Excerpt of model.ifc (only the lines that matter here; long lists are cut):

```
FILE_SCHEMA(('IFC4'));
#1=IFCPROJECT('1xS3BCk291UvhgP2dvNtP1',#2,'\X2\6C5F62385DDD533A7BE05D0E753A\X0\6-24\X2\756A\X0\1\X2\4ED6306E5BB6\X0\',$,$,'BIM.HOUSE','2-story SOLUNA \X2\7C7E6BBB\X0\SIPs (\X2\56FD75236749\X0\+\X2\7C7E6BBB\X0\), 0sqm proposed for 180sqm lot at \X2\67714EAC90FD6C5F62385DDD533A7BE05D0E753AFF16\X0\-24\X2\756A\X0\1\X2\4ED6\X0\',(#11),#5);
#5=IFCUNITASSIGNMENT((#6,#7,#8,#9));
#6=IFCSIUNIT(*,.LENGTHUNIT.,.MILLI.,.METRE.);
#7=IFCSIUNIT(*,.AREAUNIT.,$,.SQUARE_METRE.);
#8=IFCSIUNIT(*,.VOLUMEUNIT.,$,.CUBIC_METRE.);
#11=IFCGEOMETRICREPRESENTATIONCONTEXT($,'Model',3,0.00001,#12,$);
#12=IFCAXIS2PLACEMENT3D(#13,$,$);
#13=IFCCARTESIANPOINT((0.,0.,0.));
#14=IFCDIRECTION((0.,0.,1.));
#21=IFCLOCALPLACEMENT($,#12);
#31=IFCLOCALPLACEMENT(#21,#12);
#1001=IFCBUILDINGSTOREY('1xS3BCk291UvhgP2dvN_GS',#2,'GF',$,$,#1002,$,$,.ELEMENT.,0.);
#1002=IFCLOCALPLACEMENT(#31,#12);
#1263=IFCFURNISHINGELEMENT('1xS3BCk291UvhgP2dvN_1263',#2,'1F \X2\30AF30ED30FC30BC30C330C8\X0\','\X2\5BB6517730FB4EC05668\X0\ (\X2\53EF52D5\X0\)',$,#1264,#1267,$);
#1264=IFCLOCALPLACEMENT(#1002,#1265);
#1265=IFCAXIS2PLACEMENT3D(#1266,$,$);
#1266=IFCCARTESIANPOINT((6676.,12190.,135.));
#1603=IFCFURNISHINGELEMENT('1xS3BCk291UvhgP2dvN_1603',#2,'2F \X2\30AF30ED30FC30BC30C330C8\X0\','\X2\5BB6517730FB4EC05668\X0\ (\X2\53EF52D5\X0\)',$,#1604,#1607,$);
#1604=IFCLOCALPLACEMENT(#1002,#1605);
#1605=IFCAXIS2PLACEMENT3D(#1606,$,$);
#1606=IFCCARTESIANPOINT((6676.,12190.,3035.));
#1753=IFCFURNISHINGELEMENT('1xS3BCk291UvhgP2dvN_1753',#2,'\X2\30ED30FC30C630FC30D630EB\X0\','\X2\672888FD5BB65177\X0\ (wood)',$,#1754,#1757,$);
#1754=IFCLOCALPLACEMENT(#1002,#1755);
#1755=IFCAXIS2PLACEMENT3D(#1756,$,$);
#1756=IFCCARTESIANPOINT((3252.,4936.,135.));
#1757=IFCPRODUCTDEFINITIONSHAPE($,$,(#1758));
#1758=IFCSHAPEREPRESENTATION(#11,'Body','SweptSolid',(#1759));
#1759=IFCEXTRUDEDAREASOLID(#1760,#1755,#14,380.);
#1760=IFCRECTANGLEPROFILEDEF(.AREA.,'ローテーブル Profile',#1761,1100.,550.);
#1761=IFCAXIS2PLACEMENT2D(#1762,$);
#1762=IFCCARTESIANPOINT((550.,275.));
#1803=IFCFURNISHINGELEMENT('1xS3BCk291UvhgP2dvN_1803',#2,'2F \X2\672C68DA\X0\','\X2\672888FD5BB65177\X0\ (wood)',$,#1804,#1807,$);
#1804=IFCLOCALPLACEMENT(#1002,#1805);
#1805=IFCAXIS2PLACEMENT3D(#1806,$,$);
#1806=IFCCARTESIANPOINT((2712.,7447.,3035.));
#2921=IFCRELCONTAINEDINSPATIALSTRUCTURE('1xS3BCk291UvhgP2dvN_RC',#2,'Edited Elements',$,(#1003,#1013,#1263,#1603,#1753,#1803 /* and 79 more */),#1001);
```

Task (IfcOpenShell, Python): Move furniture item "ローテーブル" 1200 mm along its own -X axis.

```python
import ifcopenshell
import ifcopenshell.api.geometry
import ifcopenshell.util.placement
import ifcopenshell.util.unit

model = ifcopenshell.open("model.ifc")
unit_scale = ifcopenshell.util.unit.calculate_unit_scale(model)

item = model.by_guid("1xS3BCk291UvhgP2dvN_1753")
matrix = ifcopenshell.util.placement.get_local_placement(item.ObjectPlacement)
matrix[:3, 3] -= matrix[:3, 0] * 1.2 / unit_scale
ifcopenshell.api.geometry.edit_object_placement(model, product=item, matrix=matrix, is_si=False)

print(ifcopenshell.util.placement.get_local_placement(item.ObjectPlacement).round(3) + 0.0)

model.write("model_v2.ifc")
```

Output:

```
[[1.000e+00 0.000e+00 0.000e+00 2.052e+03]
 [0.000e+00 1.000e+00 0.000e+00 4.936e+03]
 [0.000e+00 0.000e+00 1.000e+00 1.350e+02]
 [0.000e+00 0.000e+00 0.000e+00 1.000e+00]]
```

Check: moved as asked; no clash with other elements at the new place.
